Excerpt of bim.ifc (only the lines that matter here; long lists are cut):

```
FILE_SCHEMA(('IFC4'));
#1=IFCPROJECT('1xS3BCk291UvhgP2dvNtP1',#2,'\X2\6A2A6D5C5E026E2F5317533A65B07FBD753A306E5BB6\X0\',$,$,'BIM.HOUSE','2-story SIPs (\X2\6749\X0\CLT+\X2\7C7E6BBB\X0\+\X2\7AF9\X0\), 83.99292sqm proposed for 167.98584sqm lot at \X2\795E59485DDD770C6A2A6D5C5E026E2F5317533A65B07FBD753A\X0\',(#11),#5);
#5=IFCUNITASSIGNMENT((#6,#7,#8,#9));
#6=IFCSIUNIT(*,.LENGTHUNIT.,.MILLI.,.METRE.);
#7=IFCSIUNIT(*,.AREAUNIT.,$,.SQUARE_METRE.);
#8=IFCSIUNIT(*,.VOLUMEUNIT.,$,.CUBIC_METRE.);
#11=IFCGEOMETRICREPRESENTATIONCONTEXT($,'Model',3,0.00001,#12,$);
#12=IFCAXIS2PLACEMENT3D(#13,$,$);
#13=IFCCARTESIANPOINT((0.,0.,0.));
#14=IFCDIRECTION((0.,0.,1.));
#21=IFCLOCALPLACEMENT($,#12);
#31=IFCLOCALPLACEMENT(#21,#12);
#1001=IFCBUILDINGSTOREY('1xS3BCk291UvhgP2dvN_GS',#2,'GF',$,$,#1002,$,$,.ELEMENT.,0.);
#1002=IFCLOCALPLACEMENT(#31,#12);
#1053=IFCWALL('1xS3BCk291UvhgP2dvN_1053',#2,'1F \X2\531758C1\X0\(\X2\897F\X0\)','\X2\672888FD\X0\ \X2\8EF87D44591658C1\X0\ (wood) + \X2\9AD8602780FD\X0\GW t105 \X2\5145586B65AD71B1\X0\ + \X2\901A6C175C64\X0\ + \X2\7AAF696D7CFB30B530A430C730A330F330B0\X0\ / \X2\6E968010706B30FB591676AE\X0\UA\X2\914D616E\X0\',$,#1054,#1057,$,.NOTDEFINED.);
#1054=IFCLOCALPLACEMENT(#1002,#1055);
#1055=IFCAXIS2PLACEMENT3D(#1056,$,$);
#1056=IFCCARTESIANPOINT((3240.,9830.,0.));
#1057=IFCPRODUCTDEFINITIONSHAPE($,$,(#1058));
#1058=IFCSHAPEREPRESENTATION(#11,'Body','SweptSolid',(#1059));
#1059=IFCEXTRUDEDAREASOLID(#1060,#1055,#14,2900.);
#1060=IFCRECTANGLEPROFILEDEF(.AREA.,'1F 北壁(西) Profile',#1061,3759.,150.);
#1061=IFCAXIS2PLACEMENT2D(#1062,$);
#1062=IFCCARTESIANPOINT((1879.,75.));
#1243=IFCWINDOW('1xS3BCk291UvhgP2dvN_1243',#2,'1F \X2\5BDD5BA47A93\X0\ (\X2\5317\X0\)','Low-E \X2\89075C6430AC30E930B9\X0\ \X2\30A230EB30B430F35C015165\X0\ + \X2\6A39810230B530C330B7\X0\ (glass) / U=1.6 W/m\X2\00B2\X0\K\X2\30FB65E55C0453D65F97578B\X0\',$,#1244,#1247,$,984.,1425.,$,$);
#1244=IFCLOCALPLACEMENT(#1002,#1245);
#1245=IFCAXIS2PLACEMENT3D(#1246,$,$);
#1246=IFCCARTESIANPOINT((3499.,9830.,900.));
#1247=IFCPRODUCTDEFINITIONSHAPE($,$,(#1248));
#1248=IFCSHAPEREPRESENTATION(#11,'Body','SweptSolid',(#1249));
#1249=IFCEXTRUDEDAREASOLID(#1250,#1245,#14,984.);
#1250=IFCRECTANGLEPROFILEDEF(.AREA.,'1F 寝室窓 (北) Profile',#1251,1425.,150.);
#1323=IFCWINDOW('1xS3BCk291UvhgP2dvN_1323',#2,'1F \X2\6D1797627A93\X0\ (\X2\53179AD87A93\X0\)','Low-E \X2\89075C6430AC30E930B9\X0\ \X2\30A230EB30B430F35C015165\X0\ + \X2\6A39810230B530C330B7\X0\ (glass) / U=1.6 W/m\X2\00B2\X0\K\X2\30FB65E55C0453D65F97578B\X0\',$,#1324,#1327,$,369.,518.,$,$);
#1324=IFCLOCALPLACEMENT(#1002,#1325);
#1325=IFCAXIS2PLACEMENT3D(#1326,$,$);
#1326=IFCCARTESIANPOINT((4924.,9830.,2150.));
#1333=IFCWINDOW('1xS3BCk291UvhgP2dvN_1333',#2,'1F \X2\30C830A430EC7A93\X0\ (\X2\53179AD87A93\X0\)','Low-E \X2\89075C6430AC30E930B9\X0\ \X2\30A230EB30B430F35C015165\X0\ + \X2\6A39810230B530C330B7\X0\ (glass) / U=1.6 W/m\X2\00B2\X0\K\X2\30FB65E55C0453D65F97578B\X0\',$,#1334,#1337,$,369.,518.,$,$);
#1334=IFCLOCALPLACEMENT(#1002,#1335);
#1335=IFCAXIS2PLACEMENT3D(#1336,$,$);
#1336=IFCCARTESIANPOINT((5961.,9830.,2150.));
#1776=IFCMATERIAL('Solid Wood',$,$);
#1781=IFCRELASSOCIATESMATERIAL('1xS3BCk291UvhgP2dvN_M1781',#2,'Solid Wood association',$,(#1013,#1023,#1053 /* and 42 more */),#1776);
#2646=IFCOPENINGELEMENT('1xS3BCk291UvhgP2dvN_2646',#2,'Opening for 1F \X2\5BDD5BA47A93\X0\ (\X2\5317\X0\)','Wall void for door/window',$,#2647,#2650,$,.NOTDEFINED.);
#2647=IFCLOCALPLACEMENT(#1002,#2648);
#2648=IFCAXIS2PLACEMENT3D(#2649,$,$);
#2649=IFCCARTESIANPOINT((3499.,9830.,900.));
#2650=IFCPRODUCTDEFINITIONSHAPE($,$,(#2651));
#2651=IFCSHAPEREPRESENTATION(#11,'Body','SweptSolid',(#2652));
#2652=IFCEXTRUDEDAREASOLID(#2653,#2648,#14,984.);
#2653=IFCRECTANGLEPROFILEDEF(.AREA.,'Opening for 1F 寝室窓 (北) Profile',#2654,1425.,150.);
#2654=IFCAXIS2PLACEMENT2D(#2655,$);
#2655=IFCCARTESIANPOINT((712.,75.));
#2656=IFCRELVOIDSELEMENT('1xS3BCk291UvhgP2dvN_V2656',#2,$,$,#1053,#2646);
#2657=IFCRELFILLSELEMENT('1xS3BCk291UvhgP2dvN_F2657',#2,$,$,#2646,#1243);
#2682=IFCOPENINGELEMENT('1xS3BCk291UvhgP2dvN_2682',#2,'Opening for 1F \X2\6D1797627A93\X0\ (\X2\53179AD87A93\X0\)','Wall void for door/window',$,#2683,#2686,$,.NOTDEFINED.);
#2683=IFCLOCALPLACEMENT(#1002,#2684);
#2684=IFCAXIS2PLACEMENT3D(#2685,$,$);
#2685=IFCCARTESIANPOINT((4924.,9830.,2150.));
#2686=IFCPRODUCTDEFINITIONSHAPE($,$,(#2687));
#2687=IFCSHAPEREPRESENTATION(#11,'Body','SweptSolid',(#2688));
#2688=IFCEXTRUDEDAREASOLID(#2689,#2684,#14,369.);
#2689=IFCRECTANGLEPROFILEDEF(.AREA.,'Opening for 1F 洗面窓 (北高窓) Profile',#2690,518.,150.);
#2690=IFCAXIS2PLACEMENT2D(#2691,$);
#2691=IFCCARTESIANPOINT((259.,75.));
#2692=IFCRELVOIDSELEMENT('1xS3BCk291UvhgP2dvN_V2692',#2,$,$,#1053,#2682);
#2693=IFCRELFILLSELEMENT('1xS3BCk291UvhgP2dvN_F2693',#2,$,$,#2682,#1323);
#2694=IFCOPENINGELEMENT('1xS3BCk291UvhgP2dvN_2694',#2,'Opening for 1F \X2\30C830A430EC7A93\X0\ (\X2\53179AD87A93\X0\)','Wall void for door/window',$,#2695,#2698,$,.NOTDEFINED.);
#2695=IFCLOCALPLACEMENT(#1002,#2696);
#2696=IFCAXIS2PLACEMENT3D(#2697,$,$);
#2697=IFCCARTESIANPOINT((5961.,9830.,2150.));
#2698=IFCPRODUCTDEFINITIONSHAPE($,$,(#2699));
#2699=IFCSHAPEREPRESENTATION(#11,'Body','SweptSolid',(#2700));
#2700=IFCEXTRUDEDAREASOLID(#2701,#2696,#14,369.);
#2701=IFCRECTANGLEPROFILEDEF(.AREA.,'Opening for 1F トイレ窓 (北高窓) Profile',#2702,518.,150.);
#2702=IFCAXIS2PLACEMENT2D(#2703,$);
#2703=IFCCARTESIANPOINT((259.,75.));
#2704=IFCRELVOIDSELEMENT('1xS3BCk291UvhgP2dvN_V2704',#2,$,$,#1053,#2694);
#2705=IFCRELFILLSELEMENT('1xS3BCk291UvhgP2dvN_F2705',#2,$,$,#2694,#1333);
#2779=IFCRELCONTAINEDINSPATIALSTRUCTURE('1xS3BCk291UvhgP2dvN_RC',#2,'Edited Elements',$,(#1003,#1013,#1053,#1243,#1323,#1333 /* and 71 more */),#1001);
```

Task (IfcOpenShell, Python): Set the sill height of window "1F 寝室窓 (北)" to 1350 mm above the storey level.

```python
import numpy as np
import ifcopenshell
import ifcopenshell.api.geometry
import ifcopenshell.geom
import ifcopenshell.util.element
import ifcopenshell.util.placement
import ifcopenshell.util.shape
import ifcopenshell.util.unit

model = ifcopenshell.open("bim.ifc")
unit_scale = ifcopenshell.util.unit.calculate_unit_scale(model)

window = model.by_guid("1xS3BCk291UvhgP2dvN_1243")
opening = window.FillsVoids[0].RelatingOpeningElement
storey = ifcopenshell.util.element.get_container(window, ifc_class="IfcBuildingStorey")
level = ifcopenshell.util.placement.get_local_placement(storey.ObjectPlacement)[2, 3]

# The opening's origin need not be at the sill, so measure its lowest point.
shape = ifcopenshell.geom.create_shape(ifcopenshell.geom.settings(), opening)
bottom = ifcopenshell.util.shape.get_shape_bottom_elevation(shape, shape.geometry) / unit_scale
dz = level + 1.35 / unit_scale - bottom

shift = np.array([0.0, 0.0, dz])
# The window is not placed relative to its opening, so move both.
for product in (opening, window):
    matrix = ifcopenshell.util.placement.get_local_placement(product.ObjectPlacement)
    matrix[:3, 3] += shift
    ifcopenshell.api.geometry.edit_object_placement(model, product=product, matrix=matrix, is_si=False)

print(f"moved by {dz * unit_scale:+.3f} m")

model.write("bim-out.ifc")
```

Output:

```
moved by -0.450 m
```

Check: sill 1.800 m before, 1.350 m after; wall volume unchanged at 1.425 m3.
